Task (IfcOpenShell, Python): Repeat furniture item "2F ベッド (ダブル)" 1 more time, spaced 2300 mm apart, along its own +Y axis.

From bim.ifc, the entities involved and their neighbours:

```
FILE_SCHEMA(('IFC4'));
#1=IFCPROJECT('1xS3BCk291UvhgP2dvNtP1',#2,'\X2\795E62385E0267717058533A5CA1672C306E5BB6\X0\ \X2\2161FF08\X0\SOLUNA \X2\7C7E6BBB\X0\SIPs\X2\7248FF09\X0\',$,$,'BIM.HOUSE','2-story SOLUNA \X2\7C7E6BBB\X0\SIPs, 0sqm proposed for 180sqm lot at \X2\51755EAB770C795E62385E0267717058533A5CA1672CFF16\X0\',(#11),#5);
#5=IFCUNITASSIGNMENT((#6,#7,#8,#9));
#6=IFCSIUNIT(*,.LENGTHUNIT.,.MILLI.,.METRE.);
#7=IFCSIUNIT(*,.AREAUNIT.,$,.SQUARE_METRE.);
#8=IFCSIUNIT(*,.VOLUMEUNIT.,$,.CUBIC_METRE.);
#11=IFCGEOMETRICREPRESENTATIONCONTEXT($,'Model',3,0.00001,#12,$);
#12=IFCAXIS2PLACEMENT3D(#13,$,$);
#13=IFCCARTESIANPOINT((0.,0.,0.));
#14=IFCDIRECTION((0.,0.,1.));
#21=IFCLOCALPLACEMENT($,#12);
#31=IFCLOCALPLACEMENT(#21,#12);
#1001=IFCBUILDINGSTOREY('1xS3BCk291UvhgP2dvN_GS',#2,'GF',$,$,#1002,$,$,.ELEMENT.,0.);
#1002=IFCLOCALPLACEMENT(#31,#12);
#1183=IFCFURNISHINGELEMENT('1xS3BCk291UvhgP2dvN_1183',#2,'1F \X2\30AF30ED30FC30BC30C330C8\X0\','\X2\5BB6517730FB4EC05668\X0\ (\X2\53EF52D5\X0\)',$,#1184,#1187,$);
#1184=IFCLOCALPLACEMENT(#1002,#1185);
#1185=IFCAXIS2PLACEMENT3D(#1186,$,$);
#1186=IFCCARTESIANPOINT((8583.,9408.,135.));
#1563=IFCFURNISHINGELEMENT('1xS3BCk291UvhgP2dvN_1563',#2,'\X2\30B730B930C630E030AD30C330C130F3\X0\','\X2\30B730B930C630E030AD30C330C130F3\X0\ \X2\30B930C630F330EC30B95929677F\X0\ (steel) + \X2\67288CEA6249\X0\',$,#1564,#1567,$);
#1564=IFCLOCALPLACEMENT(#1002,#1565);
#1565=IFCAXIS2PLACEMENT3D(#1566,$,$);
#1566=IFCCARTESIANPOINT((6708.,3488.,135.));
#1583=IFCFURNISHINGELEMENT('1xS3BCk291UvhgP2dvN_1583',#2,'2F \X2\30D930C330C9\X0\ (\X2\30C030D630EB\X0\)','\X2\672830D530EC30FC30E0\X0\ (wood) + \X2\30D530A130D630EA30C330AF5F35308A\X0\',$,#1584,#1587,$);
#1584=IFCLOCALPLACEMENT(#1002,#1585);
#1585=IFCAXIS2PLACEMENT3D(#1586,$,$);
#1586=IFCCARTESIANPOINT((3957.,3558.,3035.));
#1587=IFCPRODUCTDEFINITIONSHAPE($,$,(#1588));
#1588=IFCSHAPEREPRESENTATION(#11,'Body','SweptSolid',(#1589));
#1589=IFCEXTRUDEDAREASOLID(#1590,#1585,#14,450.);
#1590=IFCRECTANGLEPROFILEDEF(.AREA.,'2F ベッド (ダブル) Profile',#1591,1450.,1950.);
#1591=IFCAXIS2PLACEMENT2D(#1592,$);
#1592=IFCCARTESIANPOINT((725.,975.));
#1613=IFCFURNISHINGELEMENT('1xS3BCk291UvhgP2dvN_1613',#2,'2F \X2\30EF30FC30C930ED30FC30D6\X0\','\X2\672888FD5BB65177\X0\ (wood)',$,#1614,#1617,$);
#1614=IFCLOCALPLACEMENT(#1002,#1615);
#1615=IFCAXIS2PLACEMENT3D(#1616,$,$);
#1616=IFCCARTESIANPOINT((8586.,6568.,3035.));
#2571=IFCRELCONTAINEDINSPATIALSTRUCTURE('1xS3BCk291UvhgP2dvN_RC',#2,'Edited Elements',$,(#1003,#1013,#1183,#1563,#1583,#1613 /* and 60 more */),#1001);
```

```python
import ifcopenshell
import ifcopenshell.api.geometry
import ifcopenshell.api.root
import ifcopenshell.util.element
import ifcopenshell.util.placement

model = ifcopenshell.open("bim.ifc")


def reuse_history(source, copy):
    """copy_class also copies each property set's owner history, people and application; keep the originals."""
    for rel in copy.IsDefinedBy:
        if rel.is_a("IfcRelDefinesByProperties") and (history := rel.RelatingPropertyDefinition.OwnerHistory):
            rel.RelatingPropertyDefinition.OwnerHistory = source.OwnerHistory
            ifcopenshell.util.element.remove_deep2(model, history)


source = model.by_guid("1xS3BCk291UvhgP2dvN_1583")
base = ifcopenshell.util.placement.get_local_placement(source.ObjectPlacement)
step = base[:3, 1] * 2300.0

for i in range(1, 2):
    copy = ifcopenshell.api.root.copy_class(model, product=source)
    copy.Representation = ifcopenshell.util.element.copy_deep(
        model, source.Representation, exclude=["IfcGeometricRepresentationContext", "IfcRepresentationMap"]
    )
    reuse_history(source, copy)
    matrix = base.copy()
    matrix[:3, 3] += i * step
    print("added at", matrix[:3, 3].round(3) + 0.0)
    ifcopenshell.api.geometry.edit_object_placement(model, product=copy, matrix=matrix, is_si=False)

model.write("bim_edited.ifc")
```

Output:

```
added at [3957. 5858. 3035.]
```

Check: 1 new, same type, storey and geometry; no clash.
